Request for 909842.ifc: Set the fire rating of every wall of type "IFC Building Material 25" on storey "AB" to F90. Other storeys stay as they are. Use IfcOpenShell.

First a look at what the model holds.

```python
import ifcopenshell
import ifcopenshell.util.element

model = ifcopenshell.open("909842.ifc")
print(model.schema)
storey = next(s for s in model.by_type("IfcBuildingStorey") if s.Name == "AB")
walls = [e for e in ifcopenshell.util.element.get_decomposition(storey) if e.is_a("IfcWall")]
seen = {}
for e in walls:
    element_type = ifcopenshell.util.element.get_type(e)
    key = (element_type.Name if element_type != e and element_type else None, ifcopenshell.util.element.get_pset(e, "Pset_WallCommon", "FireRating"))
    seen[key] = seen.get(key, 0) + 1
for (name, value), count in sorted(seen.items(), key=str):
    print(count, "x", name, "|", value)
```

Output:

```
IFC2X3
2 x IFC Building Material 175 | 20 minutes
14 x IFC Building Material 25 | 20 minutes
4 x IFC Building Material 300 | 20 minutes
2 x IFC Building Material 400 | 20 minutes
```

```python
import ifcopenshell
import ifcopenshell.api.pset
import ifcopenshell.util.element

model = ifcopenshell.open("909842.ifc")

storey = next(s for s in model.by_type("IfcBuildingStorey") if s.Name == "AB")
walls = [e for e in ifcopenshell.util.element.get_decomposition(storey) if e.is_a("IfcWall")]

count = 0
for e in walls:
    element_type = ifcopenshell.util.element.get_type(e)
    if element_type in (None, e) or element_type.Name != "IFC Building Material 25":
        continue
    # add_pset returns the element's existing set when there is one.
    pset = ifcopenshell.api.pset.add_pset(model, product=e, name="Pset_WallCommon")
    ifcopenshell.api.pset.edit_pset(model, pset=pset, properties={"FireRating": "F90"})
    count += 1

print(count, "walls updated")

model.write("909842_updated.ifc")
```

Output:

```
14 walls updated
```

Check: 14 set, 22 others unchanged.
